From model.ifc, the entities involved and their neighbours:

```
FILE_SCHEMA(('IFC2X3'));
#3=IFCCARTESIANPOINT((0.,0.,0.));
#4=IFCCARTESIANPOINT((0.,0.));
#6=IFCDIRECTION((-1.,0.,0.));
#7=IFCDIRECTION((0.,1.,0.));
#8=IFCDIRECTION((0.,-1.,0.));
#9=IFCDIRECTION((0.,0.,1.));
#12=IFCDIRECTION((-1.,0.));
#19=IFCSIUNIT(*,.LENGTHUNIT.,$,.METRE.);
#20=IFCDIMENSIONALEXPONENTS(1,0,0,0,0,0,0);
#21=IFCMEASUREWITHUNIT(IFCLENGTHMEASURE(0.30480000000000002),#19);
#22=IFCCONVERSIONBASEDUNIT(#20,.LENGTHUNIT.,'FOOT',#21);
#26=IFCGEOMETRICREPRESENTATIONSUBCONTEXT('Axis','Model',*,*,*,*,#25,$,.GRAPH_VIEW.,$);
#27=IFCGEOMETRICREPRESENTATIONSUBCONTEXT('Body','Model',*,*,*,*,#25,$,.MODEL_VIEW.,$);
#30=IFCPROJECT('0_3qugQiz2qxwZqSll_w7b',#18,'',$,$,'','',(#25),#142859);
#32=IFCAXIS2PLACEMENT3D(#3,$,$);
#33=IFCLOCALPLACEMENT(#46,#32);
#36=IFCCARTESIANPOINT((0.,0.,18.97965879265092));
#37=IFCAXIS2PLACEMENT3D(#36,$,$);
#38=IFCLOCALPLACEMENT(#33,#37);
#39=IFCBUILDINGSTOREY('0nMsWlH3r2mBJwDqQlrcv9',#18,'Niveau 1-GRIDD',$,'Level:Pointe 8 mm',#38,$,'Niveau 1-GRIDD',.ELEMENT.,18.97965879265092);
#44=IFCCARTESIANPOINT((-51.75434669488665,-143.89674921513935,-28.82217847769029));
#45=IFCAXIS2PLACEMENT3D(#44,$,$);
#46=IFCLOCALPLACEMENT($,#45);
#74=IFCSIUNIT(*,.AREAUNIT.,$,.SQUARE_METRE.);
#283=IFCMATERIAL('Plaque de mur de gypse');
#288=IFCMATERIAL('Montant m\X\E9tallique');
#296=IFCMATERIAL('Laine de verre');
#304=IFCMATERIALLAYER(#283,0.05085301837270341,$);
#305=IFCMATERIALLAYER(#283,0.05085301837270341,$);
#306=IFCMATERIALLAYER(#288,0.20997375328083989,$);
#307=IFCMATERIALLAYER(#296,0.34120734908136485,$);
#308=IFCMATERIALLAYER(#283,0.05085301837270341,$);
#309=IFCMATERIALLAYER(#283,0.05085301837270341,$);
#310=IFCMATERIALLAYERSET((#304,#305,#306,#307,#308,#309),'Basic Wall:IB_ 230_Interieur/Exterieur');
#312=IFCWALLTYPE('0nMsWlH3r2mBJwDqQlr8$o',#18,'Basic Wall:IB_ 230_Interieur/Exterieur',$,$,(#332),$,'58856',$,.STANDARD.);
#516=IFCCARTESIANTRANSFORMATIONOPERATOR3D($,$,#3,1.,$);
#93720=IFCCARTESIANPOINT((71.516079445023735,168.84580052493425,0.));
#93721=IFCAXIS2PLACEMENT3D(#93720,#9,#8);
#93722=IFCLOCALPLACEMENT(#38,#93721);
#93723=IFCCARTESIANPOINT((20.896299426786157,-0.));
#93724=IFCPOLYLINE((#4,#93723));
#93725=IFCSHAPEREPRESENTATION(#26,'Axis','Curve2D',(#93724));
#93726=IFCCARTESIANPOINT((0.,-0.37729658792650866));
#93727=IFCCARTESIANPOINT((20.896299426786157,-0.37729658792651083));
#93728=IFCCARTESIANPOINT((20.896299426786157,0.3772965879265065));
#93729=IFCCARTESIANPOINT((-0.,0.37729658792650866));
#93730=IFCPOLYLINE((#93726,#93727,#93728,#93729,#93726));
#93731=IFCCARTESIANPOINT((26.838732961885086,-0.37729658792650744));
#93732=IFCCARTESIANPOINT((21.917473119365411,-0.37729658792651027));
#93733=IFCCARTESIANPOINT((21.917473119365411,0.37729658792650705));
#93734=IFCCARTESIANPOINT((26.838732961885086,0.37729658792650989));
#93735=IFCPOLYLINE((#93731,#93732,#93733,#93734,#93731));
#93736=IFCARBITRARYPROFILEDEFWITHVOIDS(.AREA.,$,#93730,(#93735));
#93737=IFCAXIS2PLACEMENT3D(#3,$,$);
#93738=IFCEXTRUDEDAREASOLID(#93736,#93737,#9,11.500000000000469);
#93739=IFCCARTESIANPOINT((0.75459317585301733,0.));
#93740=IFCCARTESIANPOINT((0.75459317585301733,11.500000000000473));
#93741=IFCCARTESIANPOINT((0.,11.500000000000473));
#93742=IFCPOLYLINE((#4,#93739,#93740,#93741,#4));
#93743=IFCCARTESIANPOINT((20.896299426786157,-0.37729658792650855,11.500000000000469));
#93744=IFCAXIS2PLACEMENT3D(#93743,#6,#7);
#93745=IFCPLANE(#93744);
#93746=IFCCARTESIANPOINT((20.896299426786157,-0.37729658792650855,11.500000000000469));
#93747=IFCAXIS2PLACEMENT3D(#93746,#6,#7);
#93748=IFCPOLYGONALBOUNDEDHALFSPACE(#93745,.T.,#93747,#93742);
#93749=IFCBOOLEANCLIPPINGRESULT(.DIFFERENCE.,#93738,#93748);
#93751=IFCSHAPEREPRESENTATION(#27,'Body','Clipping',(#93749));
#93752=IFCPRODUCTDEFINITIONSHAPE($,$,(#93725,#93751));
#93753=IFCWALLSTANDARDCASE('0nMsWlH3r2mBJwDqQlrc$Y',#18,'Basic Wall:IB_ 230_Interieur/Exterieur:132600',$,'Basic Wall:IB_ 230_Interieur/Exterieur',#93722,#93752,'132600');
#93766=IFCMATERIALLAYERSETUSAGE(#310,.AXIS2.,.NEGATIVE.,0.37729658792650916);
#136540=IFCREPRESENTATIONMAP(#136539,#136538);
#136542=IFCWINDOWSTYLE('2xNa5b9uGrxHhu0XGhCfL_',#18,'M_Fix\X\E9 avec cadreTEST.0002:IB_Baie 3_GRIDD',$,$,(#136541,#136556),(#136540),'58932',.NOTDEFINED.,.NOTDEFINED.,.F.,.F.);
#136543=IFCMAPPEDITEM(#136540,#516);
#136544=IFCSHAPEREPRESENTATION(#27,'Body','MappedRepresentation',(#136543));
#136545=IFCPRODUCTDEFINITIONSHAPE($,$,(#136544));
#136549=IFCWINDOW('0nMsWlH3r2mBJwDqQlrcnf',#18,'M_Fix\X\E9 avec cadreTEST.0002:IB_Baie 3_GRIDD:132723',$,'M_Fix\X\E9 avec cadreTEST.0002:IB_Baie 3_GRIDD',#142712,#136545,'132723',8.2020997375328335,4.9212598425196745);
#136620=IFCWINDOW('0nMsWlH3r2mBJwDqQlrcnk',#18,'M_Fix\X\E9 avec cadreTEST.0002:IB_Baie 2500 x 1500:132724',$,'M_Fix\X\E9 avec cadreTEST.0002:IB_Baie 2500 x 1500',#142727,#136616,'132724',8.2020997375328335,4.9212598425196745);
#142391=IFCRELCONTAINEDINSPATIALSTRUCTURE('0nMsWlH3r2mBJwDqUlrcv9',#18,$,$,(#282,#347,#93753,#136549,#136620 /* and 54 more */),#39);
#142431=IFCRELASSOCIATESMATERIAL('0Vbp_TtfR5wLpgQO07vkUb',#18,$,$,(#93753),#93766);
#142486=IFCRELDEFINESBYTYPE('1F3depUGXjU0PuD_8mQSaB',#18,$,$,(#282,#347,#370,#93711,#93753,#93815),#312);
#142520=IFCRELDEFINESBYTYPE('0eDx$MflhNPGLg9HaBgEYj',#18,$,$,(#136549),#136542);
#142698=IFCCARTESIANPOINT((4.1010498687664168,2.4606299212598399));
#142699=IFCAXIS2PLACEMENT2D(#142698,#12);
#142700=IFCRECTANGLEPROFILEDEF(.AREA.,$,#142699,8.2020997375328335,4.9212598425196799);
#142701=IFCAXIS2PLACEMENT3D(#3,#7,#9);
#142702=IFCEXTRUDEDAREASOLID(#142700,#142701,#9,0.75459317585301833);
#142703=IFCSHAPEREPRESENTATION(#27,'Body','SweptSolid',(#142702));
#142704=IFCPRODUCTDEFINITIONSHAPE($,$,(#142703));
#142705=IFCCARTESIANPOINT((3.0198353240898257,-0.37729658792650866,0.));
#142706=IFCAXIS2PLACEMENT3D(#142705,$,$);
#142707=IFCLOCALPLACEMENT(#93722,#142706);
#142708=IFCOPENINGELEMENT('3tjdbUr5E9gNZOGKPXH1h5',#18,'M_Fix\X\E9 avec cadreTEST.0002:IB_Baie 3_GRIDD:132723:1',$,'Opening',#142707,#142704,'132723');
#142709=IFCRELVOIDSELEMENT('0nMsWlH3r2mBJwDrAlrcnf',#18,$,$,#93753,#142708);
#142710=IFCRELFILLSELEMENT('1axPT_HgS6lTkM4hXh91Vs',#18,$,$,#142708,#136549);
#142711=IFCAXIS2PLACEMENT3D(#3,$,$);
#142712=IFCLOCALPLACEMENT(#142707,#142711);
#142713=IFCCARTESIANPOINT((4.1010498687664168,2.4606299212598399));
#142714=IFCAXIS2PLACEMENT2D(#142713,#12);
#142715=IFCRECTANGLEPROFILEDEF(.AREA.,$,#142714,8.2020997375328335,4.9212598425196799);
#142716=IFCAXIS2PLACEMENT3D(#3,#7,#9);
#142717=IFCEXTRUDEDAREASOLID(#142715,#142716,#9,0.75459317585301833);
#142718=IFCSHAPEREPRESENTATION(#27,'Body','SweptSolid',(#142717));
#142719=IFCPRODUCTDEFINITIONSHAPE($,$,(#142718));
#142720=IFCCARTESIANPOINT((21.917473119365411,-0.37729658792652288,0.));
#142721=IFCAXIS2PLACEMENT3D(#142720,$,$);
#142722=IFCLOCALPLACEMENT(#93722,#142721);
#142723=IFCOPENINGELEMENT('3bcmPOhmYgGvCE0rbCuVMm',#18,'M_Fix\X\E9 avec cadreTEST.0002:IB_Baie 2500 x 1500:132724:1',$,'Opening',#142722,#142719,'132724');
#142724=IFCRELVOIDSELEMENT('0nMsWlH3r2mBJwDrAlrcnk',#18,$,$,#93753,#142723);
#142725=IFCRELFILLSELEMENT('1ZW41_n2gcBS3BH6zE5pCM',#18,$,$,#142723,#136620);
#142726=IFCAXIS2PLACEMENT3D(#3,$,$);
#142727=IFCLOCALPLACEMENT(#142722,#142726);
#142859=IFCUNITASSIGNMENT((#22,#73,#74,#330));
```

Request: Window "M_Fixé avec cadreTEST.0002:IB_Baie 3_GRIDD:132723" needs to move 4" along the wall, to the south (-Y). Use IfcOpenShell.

```python
import ifcopenshell
import ifcopenshell.api.geometry
import ifcopenshell.util.placement
import ifcopenshell.util.unit

model = ifcopenshell.open("model.ifc")
unit_scale = ifcopenshell.util.unit.calculate_unit_scale(model)

window = model.by_guid("0nMsWlH3r2mBJwDqQlrcnf")
opening = window.FillsVoids[0].RelatingOpeningElement
wall = opening.VoidsElements[0].RelatingBuildingElement

wall_matrix = ifcopenshell.util.placement.get_local_placement(wall.ObjectPlacement)
shift = wall_matrix[:3, 0] * 4 * 0.0254 / unit_scale
before = ifcopenshell.util.placement.get_local_placement(window.ObjectPlacement)[:3, 3].copy()

# The window is placed relative to its opening, so it follows when the opening moves.
matrix = ifcopenshell.util.placement.get_local_placement(opening.ObjectPlacement)
matrix[:3, 3] += shift
ifcopenshell.api.geometry.edit_object_placement(
    model, product=opening, matrix=matrix, is_si=False, should_transform_children=True
)

after = ifcopenshell.util.placement.get_local_placement(window.ObjectPlacement)[:3, 3]
print("window moved by", (after - before).round(3) + 0.0)

model.write("model-out.ifc")
```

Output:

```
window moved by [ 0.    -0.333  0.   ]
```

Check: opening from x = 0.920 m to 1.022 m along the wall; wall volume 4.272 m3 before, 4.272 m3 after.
